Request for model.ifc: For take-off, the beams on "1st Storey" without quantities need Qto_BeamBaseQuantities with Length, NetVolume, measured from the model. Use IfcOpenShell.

First a look at what the model holds.

```python
import ifcopenshell
import ifcopenshell.util.element
import ifcopenshell.util.unit

model = ifcopenshell.open("model.ifc")
print(model.schema)
for unit_type in ("LENGTHUNIT", "AREAUNIT", "VOLUMEUNIT"):
    print(unit_type, ifcopenshell.util.unit.calculate_unit_scale(model, unit_type))
storey = next(s for s in model.by_type("IfcBuildingStorey") if s.Name == "1st Storey")
beams = [e for e in ifcopenshell.util.element.get_decomposition(storey) if e.is_a("IfcBeam")]
for e in sorted(beams, key=lambda e: e.id()):
    print(e.id(), e.is_a(), e.Name, list(ifcopenshell.util.element.get_psets(e, qtos_only=True)), sep=" | ")
```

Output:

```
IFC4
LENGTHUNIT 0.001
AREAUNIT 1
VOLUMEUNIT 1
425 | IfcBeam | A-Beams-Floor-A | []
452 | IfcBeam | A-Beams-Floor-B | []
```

```python
import ifcopenshell
import ifcopenshell.api.pset
import ifcopenshell.geom
import ifcopenshell.util.element
import ifcopenshell.util.shape
import ifcopenshell.util.unit

model = ifcopenshell.open("model.ifc")
unit_scale = ifcopenshell.util.unit.calculate_unit_scale(model)
volume_scale = ifcopenshell.util.unit.calculate_unit_scale(model, "VOLUMEUNIT")
settings = ifcopenshell.geom.settings()

storey = next(s for s in model.by_type("IfcBuildingStorey") if s.Name == "1st Storey")
beams = [e for e in ifcopenshell.util.element.get_decomposition(storey) if e.is_a("IfcBeam")]

for e in sorted(beams, key=lambda e: e.id()):
    if ifcopenshell.util.element.get_psets(e, qtos_only=True, should_inherit=False):
        continue
    # Geometry comes back in metres, in the element's own axes.
    shape = ifcopenshell.geom.create_shape(settings, e)
    values = {
        "Length": ifcopenshell.util.shape.get_max_xyz(shape.geometry) / unit_scale,
        "NetVolume": ifcopenshell.util.shape.get_volume(shape.geometry) / volume_scale,
    }
    qto = ifcopenshell.api.pset.add_qto(model, product=e, name="Qto_BeamBaseQuantities")
    ifcopenshell.api.pset.edit_qto(model, qto=qto, properties=values)
    print(e.id(), {k: round(v, 3) for k, v in values.items()})

model.write("model_v2.ifc")
```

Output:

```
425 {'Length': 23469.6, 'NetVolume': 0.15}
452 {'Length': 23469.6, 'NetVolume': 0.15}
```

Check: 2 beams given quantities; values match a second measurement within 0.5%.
